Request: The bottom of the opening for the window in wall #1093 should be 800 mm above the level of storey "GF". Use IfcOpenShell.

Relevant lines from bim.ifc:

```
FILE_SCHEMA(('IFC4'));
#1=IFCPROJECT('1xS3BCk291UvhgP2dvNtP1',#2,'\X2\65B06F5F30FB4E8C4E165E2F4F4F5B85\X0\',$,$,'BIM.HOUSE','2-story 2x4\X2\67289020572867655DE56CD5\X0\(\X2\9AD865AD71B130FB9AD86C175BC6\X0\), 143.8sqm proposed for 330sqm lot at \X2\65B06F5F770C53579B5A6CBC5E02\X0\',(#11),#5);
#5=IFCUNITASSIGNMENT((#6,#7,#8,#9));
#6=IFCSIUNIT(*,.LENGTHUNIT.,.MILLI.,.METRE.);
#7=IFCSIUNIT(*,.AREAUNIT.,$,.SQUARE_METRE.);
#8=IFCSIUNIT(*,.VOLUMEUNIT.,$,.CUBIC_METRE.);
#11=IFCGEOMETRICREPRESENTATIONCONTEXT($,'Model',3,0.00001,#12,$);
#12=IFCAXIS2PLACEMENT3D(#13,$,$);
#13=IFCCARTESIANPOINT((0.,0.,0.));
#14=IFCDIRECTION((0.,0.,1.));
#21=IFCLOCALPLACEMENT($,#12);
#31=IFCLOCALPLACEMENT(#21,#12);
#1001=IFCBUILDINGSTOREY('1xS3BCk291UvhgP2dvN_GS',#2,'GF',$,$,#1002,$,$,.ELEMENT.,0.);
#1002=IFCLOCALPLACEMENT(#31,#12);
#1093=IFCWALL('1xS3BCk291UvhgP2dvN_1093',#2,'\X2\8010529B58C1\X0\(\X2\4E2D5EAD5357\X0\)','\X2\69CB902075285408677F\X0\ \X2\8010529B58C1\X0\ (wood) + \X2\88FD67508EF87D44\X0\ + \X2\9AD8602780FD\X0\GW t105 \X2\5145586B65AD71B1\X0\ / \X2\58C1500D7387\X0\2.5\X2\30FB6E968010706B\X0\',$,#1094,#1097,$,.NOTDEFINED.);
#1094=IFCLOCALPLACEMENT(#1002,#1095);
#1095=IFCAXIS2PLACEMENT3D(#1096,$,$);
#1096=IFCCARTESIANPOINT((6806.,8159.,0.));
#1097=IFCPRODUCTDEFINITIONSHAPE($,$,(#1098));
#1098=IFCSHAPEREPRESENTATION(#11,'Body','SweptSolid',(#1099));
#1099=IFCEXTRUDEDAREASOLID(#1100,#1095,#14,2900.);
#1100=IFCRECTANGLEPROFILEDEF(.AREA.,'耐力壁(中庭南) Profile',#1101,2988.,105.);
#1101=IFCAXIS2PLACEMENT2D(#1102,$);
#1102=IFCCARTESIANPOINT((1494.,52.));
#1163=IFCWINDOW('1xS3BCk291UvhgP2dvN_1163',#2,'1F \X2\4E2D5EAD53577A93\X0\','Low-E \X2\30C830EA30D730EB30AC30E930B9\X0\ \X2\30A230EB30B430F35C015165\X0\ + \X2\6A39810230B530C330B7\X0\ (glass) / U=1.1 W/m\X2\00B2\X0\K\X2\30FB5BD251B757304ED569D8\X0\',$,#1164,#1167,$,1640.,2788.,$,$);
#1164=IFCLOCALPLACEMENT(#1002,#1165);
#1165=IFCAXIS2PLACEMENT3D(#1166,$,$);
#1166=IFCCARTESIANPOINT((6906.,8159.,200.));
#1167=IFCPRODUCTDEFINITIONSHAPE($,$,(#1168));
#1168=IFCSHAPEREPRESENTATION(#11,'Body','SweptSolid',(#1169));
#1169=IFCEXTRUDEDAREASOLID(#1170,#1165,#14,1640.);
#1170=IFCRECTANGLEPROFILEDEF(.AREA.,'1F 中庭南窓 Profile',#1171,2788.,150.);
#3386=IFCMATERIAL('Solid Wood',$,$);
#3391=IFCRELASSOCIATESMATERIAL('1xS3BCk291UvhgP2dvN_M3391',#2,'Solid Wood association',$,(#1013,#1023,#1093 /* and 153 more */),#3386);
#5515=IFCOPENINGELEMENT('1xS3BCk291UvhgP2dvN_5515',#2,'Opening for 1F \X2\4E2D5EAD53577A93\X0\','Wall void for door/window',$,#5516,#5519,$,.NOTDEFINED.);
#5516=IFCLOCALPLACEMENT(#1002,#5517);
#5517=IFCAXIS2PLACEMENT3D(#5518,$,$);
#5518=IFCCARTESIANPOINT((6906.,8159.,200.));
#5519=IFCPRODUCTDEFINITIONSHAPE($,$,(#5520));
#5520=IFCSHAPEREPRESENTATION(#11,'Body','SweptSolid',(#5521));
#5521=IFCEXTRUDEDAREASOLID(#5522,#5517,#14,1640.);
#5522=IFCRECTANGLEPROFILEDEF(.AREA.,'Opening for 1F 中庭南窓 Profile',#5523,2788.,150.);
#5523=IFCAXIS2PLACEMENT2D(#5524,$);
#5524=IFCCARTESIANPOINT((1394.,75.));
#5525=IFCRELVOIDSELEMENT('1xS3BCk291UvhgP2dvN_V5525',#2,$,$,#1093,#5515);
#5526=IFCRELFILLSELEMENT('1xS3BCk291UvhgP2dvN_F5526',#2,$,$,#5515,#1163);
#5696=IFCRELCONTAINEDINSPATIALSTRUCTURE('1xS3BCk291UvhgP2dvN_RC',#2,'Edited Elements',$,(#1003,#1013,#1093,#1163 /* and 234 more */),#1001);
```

```python
import numpy as np
import ifcopenshell
import ifcopenshell.api.geometry
import ifcopenshell.geom
import ifcopenshell.util.element
import ifcopenshell.util.placement
import ifcopenshell.util.shape
import ifcopenshell.util.unit

model = ifcopenshell.open("bim.ifc")
unit_scale = ifcopenshell.util.unit.calculate_unit_scale(model)

window = model.by_id(1163)
opening = window.FillsVoids[0].RelatingOpeningElement
storey = ifcopenshell.util.element.get_container(window, ifc_class="IfcBuildingStorey")
level = ifcopenshell.util.placement.get_local_placement(storey.ObjectPlacement)[2, 3]

# The opening's origin need not be at the sill, so measure its lowest point.
shape = ifcopenshell.geom.create_shape(ifcopenshell.geom.settings(), opening)
bottom = ifcopenshell.util.shape.get_shape_bottom_elevation(shape, shape.geometry) / unit_scale
dz = level + 800.0 - bottom

shift = np.array([0.0, 0.0, dz])
# The window is not placed relative to its opening, so move both.
for product in (opening, window):
    matrix = ifcopenshell.util.placement.get_local_placement(product.ObjectPlacement)
    matrix[:3, 3] += shift
    ifcopenshell.api.geometry.edit_object_placement(model, product=product, matrix=matrix, is_si=False)

print(f"moved by {dz * unit_scale:+.3f} m")

model.write("bim_v2.ifc")
```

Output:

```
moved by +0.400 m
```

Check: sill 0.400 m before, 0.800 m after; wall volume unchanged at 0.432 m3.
